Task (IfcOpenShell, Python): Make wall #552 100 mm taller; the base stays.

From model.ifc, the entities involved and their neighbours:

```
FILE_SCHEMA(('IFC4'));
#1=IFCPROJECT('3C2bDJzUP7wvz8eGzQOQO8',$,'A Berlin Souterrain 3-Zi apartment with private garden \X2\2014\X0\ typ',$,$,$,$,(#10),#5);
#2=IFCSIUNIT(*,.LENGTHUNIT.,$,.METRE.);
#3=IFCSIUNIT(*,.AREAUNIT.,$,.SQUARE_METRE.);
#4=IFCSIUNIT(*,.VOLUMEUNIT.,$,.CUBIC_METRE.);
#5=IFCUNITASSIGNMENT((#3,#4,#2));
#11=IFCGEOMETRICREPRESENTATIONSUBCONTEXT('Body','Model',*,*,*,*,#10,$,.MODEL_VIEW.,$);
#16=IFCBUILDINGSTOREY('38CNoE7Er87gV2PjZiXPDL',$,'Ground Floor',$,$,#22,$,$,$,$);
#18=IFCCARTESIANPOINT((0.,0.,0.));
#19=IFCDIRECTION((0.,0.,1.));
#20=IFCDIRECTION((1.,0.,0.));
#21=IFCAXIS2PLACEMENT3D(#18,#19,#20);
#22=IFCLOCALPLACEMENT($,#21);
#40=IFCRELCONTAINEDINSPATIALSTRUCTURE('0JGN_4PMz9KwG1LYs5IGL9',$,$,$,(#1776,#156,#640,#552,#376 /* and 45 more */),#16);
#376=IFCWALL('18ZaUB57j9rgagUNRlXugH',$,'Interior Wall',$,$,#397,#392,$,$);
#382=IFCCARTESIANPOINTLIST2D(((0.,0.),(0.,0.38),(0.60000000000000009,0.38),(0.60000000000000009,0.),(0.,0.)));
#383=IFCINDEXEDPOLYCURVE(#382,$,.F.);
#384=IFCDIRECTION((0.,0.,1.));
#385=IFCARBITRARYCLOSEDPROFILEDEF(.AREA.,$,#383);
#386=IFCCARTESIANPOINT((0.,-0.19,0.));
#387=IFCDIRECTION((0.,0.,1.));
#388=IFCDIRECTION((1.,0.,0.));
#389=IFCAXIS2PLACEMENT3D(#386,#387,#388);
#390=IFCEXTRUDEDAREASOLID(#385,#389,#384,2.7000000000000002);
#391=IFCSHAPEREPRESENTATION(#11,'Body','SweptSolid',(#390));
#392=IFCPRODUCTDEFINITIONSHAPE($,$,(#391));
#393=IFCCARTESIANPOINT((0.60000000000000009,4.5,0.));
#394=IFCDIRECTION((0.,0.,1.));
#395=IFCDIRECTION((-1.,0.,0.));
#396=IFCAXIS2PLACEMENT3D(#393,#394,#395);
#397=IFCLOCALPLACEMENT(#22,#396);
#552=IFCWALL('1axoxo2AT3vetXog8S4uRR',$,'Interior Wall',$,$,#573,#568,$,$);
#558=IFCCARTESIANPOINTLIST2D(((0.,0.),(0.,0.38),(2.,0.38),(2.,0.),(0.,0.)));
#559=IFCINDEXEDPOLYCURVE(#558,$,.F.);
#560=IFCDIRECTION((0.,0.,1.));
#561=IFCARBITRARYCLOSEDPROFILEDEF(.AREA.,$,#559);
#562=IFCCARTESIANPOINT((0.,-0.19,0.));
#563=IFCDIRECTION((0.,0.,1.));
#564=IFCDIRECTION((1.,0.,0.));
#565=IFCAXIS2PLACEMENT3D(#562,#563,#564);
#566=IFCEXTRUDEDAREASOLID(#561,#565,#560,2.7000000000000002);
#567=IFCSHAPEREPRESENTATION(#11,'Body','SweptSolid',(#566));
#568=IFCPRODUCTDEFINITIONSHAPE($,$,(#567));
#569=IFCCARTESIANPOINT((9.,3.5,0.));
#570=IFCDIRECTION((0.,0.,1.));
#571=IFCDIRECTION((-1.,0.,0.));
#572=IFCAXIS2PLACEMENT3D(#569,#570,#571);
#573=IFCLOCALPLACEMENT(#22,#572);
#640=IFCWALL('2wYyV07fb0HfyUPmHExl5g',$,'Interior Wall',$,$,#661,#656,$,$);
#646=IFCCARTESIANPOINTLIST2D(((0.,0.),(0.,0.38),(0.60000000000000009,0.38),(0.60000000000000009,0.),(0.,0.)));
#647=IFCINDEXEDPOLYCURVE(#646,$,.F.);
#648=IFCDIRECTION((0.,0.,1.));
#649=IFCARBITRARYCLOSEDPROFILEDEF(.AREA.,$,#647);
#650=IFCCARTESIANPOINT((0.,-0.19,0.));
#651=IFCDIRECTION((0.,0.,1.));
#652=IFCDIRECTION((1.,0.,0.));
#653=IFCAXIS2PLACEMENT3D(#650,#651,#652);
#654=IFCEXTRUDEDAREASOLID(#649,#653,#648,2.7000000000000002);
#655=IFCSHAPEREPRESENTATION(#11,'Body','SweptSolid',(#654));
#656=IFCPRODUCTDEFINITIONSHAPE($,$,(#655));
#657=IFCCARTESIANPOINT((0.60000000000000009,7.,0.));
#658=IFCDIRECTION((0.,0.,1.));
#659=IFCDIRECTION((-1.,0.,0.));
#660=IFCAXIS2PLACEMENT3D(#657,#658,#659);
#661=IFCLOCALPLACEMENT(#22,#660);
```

```python
import ifcopenshell
import ifcopenshell.geom
import ifcopenshell.util.representation
import ifcopenshell.util.shape

model = ifcopenshell.open("model.ifc")
settings = ifcopenshell.geom.settings()


def volume(element):
    """Net volume in cubic metres, openings subtracted."""
    shape = ifcopenshell.geom.create_shape(settings, element)
    return ifcopenshell.util.shape.get_volume(shape.geometry)


wall = model.by_id(552)
before = volume(wall)

body = ifcopenshell.util.representation.get_representation(wall, "Model", "Body")
solid = body.Items[0]
old_height = solid.Depth
solid.Depth += 0.1
after = volume(wall)

print(f"height {old_height:g} -> {solid.Depth:g}, volume {before:.3f} -> {after:.3f} m3")

model.write("model-out.ifc")
```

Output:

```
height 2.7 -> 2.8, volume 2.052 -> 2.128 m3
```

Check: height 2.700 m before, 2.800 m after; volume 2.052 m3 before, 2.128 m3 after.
